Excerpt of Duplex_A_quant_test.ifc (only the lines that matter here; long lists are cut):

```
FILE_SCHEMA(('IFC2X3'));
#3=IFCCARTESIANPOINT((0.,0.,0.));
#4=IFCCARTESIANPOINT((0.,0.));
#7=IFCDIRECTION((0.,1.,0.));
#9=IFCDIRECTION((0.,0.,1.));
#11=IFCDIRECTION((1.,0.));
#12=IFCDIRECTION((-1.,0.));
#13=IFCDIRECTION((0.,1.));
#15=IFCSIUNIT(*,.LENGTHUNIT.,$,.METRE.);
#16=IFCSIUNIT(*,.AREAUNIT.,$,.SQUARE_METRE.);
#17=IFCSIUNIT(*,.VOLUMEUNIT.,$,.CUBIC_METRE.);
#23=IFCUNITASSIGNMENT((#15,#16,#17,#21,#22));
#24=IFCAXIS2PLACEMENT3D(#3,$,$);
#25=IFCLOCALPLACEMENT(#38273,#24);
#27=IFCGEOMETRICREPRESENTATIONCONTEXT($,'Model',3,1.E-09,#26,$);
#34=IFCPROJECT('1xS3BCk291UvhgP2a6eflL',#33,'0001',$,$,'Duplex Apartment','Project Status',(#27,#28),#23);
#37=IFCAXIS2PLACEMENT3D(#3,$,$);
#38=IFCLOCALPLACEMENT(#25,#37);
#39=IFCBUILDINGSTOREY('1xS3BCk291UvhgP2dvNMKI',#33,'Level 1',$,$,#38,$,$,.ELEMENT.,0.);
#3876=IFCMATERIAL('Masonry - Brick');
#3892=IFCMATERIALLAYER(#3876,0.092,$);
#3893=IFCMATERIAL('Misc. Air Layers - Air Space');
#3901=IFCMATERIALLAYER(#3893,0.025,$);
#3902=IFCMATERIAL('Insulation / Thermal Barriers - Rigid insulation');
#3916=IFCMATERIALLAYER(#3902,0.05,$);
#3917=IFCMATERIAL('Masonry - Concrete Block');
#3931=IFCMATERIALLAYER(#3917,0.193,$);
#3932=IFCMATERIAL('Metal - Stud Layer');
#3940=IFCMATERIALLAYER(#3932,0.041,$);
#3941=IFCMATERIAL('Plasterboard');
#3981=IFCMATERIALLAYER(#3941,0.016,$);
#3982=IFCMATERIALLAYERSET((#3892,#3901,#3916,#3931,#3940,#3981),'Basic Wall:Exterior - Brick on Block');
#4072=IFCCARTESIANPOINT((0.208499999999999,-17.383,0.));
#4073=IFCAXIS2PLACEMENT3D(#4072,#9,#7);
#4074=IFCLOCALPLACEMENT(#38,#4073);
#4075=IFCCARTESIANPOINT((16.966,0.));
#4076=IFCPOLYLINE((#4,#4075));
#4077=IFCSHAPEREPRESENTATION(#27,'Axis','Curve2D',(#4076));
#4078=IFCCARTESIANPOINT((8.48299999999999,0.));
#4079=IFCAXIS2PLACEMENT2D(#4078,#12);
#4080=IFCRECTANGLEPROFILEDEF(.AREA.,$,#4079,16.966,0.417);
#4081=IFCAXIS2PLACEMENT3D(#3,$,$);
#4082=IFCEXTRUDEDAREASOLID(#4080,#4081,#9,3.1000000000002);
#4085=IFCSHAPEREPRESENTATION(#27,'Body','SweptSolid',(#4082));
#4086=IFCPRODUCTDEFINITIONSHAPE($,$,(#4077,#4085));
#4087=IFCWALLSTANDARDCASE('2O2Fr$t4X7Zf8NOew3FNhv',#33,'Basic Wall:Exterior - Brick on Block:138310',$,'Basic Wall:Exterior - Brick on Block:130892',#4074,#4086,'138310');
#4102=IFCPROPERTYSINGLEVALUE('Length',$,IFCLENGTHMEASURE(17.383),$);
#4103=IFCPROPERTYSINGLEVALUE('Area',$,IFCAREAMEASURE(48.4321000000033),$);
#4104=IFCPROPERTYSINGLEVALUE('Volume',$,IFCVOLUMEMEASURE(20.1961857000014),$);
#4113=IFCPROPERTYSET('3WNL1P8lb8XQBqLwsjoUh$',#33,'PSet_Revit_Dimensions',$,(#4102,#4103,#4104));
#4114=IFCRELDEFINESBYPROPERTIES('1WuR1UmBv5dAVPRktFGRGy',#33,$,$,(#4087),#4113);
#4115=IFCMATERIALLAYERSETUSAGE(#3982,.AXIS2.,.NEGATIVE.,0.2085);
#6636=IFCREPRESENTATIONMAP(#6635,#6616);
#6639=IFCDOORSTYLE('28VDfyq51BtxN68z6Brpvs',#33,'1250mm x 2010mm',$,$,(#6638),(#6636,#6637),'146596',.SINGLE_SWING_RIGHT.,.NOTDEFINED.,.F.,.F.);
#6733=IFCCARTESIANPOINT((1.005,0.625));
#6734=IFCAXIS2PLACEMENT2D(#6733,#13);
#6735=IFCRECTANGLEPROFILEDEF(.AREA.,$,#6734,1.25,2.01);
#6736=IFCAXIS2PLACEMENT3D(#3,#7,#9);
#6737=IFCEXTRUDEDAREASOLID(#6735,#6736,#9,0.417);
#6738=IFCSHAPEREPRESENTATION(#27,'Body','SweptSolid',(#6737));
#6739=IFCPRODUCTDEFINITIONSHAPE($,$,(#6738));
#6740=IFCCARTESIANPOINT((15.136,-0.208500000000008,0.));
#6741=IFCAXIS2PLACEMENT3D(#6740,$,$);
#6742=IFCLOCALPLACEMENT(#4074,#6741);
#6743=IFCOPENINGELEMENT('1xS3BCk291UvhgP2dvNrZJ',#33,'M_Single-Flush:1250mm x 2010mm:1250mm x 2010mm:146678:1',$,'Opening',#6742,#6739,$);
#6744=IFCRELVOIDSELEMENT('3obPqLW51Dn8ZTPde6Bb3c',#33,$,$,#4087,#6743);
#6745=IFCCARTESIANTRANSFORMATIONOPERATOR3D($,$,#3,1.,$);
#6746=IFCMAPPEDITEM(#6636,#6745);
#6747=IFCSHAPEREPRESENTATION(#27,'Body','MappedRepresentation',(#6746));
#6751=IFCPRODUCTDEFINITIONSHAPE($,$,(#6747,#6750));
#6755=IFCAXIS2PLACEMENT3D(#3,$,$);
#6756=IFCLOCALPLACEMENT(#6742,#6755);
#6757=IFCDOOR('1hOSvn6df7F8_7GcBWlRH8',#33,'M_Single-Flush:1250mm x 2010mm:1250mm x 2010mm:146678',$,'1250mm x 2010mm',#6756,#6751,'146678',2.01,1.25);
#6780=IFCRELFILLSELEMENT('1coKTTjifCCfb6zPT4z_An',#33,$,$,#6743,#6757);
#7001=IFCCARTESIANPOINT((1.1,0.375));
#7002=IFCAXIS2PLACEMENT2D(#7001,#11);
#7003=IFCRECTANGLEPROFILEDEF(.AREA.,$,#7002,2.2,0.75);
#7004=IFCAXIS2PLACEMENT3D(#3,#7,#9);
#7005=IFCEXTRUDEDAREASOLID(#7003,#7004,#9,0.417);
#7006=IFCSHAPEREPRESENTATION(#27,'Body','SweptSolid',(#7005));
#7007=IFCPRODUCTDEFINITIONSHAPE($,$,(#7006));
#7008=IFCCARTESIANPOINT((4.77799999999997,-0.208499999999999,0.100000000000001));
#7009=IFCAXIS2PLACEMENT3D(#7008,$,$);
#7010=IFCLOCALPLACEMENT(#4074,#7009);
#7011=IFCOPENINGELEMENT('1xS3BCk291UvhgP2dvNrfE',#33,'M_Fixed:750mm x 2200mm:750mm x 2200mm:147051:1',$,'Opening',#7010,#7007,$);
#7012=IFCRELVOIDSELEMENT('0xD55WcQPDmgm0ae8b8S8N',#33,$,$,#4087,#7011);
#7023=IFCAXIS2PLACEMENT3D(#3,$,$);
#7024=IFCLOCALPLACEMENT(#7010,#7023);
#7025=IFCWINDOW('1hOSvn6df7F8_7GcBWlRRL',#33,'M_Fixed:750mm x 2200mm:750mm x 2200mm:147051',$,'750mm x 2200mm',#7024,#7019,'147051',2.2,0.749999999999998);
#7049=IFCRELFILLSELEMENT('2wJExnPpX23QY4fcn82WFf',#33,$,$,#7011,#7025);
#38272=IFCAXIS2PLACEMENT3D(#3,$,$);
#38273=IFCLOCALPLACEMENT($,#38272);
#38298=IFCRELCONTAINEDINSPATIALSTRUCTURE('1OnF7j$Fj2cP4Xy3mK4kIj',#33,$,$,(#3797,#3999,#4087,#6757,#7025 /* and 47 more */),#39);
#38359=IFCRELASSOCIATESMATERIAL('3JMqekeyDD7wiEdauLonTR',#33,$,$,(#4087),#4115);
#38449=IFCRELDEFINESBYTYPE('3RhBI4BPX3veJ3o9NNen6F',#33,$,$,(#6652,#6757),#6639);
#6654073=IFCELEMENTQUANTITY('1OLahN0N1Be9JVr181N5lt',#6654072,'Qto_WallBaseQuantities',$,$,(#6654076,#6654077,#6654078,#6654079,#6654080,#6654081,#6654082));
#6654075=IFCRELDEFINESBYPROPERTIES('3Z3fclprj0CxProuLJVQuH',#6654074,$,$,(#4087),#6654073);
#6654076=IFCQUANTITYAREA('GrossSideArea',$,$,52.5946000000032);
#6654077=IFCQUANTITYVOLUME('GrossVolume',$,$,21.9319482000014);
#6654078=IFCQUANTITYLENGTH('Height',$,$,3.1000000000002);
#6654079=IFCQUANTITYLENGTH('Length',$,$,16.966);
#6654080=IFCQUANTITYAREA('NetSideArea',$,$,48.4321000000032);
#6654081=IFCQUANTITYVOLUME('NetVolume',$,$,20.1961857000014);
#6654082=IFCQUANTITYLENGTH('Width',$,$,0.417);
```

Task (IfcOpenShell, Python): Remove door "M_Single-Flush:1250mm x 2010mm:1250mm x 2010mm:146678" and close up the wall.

```python
import ifcopenshell
import ifcopenshell.api.feature
import ifcopenshell.api.pset
import ifcopenshell.api.root
import ifcopenshell.geom
import ifcopenshell.util.element
import ifcopenshell.util.shape
import ifcopenshell.util.unit

model = ifcopenshell.open("Duplex_A_quant_test.ifc")
area_scale = ifcopenshell.util.unit.calculate_unit_scale(model, "AREAUNIT")
volume_scale = ifcopenshell.util.unit.calculate_unit_scale(model, "VOLUMEUNIT")
settings = ifcopenshell.geom.settings()


def volume(element):
    """Net volume in cubic metres, openings subtracted."""
    shape = ifcopenshell.geom.create_shape(settings, element)
    return ifcopenshell.util.shape.get_volume(shape.geometry)


door = model.by_id(6757)
opening = door.FillsVoids[0].RelatingOpeningElement
wall = opening.VoidsElements[0].RelatingBuildingElement
before = volume(wall)

ifcopenshell.api.root.remove_product(model, product=door)
ifcopenshell.api.feature.remove_feature(model, feature=opening)

after = volume(wall)
thickness = 0.417  # wall thickness in metres

# Update the wall's stored quantities.
pset = model.by_id(ifcopenshell.util.element.get_pset(wall, "PSet_Revit_Dimensions", should_inherit=False)["id"])
ifcopenshell.api.pset.edit_pset(model, pset=pset, properties={
    "Area": model.create_entity("IfcAreaMeasure", after / thickness / area_scale),
    "Volume": model.create_entity("IfcVolumeMeasure", after / volume_scale),
})
qto = model.by_id(ifcopenshell.util.element.get_pset(wall, "Qto_WallBaseQuantities", should_inherit=False)["id"])
ifcopenshell.api.pset.edit_qto(model, qto=qto, properties={
    "NetSideArea": after / thickness / area_scale,
    "NetVolume": after / volume_scale,
})

print(f"wall volume {before:.3f} -> {after:.3f} m3")

model.write("Duplex_A_quant_test_edited.ifc")
```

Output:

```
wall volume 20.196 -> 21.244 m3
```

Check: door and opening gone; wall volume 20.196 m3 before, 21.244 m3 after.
